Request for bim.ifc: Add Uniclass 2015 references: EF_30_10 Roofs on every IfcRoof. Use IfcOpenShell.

First a look at what the model holds.

```python
import ifcopenshell

model = ifcopenshell.open("bim.ifc")
print(model.schema)
print("classifications:", [c.Name for c in model.by_type("IfcClassification")])
for ifc_class in ("IfcDoor", "IfcRoof", "IfcStair", "IfcWall", "IfcWindow"):
    print(ifc_class, len(model.by_type(ifc_class)))
```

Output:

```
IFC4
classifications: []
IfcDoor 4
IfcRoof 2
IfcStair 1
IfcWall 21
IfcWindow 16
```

```python
import ifcopenshell
import ifcopenshell.api.classification

model = ifcopenshell.open("bim.ifc")

system = ifcopenshell.api.classification.add_classification(model, classification="Uniclass 2015")

codes = {
    "IfcRoof": ("EF_30_10", "Roofs"),
}
for ifc_class, (code, name) in codes.items():
    products = model.by_type(ifc_class)
    ifcopenshell.api.classification.add_reference(
        model, products=products, classification=system, identification=code, name=name
    )
    print(code, len(products))

model.write("bim_updated.ifc")
```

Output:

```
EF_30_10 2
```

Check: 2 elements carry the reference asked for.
